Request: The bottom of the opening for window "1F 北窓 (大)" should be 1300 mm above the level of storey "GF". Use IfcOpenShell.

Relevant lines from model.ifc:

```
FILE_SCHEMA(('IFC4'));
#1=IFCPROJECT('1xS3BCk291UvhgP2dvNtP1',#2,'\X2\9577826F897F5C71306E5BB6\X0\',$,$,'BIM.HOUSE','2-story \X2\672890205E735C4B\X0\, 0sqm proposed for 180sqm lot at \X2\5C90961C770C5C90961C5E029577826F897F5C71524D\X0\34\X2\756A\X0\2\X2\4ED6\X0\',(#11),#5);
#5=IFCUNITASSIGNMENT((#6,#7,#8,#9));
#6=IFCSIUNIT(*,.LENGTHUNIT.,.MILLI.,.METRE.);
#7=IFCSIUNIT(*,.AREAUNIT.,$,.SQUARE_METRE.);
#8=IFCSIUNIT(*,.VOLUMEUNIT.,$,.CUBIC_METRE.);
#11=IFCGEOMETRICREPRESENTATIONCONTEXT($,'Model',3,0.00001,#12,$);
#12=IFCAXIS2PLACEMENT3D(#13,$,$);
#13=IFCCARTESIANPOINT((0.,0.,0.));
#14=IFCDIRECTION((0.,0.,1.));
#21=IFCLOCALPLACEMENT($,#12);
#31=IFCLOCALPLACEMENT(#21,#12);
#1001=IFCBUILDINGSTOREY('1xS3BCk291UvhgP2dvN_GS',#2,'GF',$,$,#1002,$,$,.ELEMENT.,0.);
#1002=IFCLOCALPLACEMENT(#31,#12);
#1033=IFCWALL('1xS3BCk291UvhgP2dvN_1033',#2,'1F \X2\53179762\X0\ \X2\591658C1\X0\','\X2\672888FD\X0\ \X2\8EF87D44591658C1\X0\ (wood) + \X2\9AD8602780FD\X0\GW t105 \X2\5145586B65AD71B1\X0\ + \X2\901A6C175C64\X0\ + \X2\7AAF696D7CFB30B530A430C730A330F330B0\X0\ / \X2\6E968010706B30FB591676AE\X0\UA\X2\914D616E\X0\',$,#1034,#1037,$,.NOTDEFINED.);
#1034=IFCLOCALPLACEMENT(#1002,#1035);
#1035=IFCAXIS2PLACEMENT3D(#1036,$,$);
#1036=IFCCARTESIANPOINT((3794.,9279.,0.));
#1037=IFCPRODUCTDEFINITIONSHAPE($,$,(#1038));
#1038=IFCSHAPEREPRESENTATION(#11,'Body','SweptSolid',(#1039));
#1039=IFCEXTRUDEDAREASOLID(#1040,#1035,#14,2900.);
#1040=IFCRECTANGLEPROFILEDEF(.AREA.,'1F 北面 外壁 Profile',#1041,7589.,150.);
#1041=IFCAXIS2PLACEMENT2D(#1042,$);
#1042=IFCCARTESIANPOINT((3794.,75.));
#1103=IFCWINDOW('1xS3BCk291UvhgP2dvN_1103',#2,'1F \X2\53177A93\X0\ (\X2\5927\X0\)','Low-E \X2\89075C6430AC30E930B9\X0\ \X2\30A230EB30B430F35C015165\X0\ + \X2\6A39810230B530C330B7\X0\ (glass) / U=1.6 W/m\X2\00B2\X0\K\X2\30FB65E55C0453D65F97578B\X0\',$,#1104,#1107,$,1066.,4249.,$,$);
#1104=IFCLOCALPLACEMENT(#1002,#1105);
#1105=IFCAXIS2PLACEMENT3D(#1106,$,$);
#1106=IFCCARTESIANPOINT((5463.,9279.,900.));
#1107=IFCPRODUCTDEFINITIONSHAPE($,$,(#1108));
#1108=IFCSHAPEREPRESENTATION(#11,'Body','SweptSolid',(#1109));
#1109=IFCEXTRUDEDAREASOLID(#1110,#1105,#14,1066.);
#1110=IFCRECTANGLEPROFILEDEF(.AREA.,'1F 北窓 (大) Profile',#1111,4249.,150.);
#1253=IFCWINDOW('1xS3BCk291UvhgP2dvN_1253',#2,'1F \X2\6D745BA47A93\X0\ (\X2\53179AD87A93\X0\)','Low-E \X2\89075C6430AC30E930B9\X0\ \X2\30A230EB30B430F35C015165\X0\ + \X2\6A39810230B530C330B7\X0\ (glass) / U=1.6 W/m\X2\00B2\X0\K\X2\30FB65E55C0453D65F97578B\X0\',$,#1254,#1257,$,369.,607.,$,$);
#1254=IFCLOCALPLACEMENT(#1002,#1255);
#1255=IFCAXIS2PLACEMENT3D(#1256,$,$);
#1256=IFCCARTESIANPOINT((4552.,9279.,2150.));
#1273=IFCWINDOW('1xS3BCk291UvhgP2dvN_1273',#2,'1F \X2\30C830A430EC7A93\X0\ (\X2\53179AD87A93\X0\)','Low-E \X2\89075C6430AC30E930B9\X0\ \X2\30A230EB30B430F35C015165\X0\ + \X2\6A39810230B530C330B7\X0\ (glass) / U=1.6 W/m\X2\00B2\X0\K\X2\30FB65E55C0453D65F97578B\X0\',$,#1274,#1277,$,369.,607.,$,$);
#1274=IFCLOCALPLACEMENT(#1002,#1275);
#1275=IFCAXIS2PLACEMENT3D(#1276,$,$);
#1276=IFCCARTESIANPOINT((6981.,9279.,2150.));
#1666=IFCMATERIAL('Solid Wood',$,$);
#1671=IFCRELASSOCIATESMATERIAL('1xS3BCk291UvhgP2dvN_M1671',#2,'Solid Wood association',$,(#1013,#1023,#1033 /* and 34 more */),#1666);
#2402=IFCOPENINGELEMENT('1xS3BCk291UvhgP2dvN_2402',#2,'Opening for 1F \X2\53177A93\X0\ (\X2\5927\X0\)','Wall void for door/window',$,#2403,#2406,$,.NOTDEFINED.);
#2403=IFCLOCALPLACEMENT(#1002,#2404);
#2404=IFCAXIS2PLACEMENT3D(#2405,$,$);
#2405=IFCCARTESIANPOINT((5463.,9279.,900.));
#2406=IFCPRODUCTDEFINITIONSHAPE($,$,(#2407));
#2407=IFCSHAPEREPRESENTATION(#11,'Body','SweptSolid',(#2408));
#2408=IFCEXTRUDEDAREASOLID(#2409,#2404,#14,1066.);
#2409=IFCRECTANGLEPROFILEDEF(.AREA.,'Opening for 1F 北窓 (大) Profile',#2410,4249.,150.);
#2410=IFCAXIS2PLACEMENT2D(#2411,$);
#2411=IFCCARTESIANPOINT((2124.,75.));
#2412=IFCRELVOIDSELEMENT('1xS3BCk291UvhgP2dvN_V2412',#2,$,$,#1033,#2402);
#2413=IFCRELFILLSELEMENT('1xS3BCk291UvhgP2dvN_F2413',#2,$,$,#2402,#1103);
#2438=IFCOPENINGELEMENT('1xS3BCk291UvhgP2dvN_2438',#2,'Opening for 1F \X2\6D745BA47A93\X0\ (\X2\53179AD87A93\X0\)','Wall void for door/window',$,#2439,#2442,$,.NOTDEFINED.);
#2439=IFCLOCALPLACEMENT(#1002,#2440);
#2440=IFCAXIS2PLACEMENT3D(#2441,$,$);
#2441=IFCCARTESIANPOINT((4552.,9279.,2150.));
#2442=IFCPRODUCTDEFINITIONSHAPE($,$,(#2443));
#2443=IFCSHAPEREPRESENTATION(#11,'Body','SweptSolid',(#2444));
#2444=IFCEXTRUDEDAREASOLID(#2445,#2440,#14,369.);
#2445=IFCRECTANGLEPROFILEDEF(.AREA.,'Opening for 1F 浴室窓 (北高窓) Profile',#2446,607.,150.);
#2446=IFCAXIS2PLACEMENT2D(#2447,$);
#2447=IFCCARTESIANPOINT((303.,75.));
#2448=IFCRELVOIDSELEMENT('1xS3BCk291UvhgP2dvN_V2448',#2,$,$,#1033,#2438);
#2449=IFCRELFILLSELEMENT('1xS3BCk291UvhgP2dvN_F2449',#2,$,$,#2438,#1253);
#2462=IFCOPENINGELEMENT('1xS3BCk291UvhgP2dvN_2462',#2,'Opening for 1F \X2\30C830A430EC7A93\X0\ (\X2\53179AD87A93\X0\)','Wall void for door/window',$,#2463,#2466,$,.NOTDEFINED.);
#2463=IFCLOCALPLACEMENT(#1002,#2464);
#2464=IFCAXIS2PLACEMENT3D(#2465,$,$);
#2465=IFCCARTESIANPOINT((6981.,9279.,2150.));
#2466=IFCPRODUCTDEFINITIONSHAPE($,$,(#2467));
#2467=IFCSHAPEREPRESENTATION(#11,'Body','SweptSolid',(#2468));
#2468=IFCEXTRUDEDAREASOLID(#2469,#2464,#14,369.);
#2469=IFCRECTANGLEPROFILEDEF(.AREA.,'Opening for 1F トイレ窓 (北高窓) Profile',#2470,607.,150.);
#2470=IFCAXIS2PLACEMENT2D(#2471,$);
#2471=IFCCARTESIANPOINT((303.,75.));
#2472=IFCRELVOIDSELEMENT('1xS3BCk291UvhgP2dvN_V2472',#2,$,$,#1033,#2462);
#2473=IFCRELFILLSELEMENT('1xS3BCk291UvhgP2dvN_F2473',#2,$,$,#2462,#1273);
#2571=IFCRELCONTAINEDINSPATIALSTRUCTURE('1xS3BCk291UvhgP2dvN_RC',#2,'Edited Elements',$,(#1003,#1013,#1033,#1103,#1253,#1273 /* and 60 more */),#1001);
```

```python
import numpy as np
import ifcopenshell
import ifcopenshell.api.geometry
import ifcopenshell.geom
import ifcopenshell.util.element
import ifcopenshell.util.placement
import ifcopenshell.util.shape
import ifcopenshell.util.unit

model = ifcopenshell.open("model.ifc")
unit_scale = ifcopenshell.util.unit.calculate_unit_scale(model)

window = model.by_guid("1xS3BCk291UvhgP2dvN_1103")
opening = window.FillsVoids[0].RelatingOpeningElement
storey = ifcopenshell.util.element.get_container(window, ifc_class="IfcBuildingStorey")
level = ifcopenshell.util.placement.get_local_placement(storey.ObjectPlacement)[2, 3]

# The opening's origin need not be at the sill, so measure its lowest point.
shape = ifcopenshell.geom.create_shape(ifcopenshell.geom.settings(), opening)
bottom = ifcopenshell.util.shape.get_shape_bottom_elevation(shape, shape.geometry) / unit_scale
dz = level + 1300.0 - bottom

shift = np.array([0.0, 0.0, dz])
# The window is not placed relative to its opening, so move both.
for product in (opening, window):
    matrix = ifcopenshell.util.placement.get_local_placement(product.ObjectPlacement)
    matrix[:3, 3] += shift
    ifcopenshell.api.geometry.edit_object_placement(model, product=product, matrix=matrix, is_si=False)

print(f"moved by {dz * unit_scale:+.3f} m")

model.write("model-out.ifc")
```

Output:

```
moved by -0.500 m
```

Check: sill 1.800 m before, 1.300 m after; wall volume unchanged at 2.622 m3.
